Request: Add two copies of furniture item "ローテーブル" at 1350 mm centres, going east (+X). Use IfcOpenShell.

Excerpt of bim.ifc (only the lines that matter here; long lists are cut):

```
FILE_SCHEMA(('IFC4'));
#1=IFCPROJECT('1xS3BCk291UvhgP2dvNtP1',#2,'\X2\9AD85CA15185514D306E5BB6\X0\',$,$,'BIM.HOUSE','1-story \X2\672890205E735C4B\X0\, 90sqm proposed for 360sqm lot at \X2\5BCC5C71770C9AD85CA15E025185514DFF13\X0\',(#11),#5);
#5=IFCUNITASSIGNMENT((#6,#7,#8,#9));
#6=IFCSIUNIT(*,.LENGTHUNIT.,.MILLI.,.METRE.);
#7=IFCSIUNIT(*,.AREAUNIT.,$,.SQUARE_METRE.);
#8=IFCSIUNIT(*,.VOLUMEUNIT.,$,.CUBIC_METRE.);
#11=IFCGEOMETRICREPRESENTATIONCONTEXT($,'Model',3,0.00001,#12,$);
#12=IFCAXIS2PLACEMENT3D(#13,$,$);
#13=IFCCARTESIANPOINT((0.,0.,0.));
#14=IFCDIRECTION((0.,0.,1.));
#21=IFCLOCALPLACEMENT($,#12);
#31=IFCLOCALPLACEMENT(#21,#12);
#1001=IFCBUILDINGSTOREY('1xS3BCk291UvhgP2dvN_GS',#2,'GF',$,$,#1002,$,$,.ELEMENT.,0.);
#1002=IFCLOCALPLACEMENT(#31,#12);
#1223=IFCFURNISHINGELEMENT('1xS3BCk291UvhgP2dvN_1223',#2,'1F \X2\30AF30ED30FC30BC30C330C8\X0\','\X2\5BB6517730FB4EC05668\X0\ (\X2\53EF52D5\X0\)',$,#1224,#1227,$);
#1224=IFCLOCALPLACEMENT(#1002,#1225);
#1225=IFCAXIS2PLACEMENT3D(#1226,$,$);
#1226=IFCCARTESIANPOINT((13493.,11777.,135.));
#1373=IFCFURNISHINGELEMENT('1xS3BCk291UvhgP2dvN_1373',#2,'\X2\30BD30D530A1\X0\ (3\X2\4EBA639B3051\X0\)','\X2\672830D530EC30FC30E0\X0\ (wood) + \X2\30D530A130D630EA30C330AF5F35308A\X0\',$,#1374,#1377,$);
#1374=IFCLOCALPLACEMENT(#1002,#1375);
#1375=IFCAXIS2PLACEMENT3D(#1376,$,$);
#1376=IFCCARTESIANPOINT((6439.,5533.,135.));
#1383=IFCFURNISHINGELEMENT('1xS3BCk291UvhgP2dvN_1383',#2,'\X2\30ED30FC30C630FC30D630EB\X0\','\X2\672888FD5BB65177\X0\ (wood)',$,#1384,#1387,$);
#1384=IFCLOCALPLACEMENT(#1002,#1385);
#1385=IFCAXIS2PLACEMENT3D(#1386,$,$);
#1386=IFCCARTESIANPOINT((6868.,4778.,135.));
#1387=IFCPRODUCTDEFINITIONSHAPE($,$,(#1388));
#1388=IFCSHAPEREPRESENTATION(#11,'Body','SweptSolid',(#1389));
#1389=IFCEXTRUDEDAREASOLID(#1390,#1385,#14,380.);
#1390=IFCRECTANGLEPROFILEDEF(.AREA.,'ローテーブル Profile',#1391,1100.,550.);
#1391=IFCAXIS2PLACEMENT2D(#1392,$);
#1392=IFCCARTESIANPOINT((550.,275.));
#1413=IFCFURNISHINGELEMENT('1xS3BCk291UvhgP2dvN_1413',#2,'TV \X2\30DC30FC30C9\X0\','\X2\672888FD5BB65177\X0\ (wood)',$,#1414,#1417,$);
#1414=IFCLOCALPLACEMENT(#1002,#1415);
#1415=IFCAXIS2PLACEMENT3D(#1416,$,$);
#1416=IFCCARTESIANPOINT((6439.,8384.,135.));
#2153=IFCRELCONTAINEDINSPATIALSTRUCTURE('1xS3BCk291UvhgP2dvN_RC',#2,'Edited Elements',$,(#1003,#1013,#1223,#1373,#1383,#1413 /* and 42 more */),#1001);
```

```python
import numpy as np
import ifcopenshell
import ifcopenshell.api.geometry
import ifcopenshell.api.root
import ifcopenshell.util.element
import ifcopenshell.util.placement

model = ifcopenshell.open("bim.ifc")


def reuse_history(source, copy):
    """copy_class also copies each property set's owner history, people and application; keep the originals."""
    for rel in copy.IsDefinedBy:
        if rel.is_a("IfcRelDefinesByProperties") and (history := rel.RelatingPropertyDefinition.OwnerHistory):
            rel.RelatingPropertyDefinition.OwnerHistory = source.OwnerHistory
            ifcopenshell.util.element.remove_deep2(model, history)


source = model.by_guid("1xS3BCk291UvhgP2dvN_1383")
base = ifcopenshell.util.placement.get_local_placement(source.ObjectPlacement)
step = np.array([1.0, 0.0, 0.0]) * 1350.0

for i in range(1, 3):
    copy = ifcopenshell.api.root.copy_class(model, product=source)
    copy.Representation = ifcopenshell.util.element.copy_deep(
        model, source.Representation, exclude=["IfcGeometricRepresentationContext", "IfcRepresentationMap"]
    )
    reuse_history(source, copy)
    matrix = base.copy()
    matrix[:3, 3] += i * step
    print("added at", matrix[:3, 3].round(3) + 0.0)
    ifcopenshell.api.geometry.edit_object_placement(model, product=copy, matrix=matrix, is_si=False)

model.write("bim_rev.ifc")
```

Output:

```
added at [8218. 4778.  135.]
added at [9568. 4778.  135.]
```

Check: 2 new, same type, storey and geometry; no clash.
